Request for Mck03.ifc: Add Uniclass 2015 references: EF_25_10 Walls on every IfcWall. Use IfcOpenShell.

First a look at what the model holds.

```python
import ifcopenshell

model = ifcopenshell.open("Mck03.ifc")
print(model.schema)
print("classifications:", [c.Name for c in model.by_type("IfcClassification")])
for ifc_class in ("IfcDoor", "IfcRoof", "IfcStair", "IfcWall", "IfcWindow"):
    print(ifc_class, len(model.by_type(ifc_class)))
```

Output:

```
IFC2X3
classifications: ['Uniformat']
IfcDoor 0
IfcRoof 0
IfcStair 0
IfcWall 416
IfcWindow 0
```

```python
import ifcopenshell
import ifcopenshell.api.classification

model = ifcopenshell.open("Mck03.ifc")

# IFC2X3 requires Source and Edition and has no link from the project to the system.
system = model.create_entity("IfcClassification", Source="NBS", Edition="2015", Name="Uniclass 2015")

codes = {
    "IfcWall": ("EF_25_10", "Walls"),
}
for ifc_class, (code, name) in codes.items():
    products = model.by_type(ifc_class)
    ifcopenshell.api.classification.add_reference(
        model, products=products, classification=system, identification=code, name=name
    )
    print(code, len(products))

model.write("Mck03_edited.ifc")
```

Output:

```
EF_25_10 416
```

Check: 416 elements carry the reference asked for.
